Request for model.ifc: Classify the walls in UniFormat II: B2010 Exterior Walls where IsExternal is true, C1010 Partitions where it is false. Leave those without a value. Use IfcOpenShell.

First a look at what the model holds.

```python
import ifcopenshell
import ifcopenshell.util.element

model = ifcopenshell.open("model.ifc")
print(model.schema)
print("classifications:", [c.Name for c in model.by_type("IfcClassification")])
values = [ifcopenshell.util.element.get_pset(e, "Pset_WallCommon", "IsExternal") for e in model.by_type("IfcWall")]
for value in (True, False, None):
    print("IsExternal", value, values.count(value))
```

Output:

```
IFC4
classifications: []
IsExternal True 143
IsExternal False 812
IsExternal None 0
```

```python
import ifcopenshell
import ifcopenshell.api.classification
import ifcopenshell.util.element

model = ifcopenshell.open("model.ifc")

system = ifcopenshell.api.classification.add_classification(model, classification="UniFormat II")

walls = model.by_type("IfcWall")
external = {e: ifcopenshell.util.element.get_pset(e, "Pset_WallCommon", "IsExternal") for e in walls}
for flag, code, name in ((True, "B2010", "Exterior Walls"), (False, "C1010", "Partitions")):
    products = [e for e in walls if external[e] is flag]
    ifcopenshell.api.classification.add_reference(
        model, products=products, classification=system, identification=code, name=name
    )
    print(code, len(products))

model.write("model_updated.ifc")
```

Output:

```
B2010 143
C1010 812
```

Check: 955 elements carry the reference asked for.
